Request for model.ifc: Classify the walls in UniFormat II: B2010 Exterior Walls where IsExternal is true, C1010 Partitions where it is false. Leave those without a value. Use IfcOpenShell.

First a look at what the model holds.

```python
import ifcopenshell
import ifcopenshell.util.element

model = ifcopenshell.open("model.ifc")
print(model.schema)
print("classifications:", [c.Name for c in model.by_type("IfcClassification")])
values = [ifcopenshell.util.element.get_pset(e, "Pset_WallCommon", "IsExternal") for e in model.by_type("IfcWall")]
for value in (True, False, None):
    print("IsExternal", value, values.count(value))
```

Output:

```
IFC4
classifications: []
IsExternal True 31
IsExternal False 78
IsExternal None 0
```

```python
import ifcopenshell
import ifcopenshell.api.classification
import ifcopenshell.util.element

model = ifcopenshell.open("model.ifc")

system = ifcopenshell.api.classification.add_classification(model, classification="UniFormat II")

walls = model.by_type("IfcWall")
external = {e: ifcopenshell.util.element.get_pset(e, "Pset_WallCommon", "IsExternal") for e in walls}
for flag, code, name in ((True, "B2010", "Exterior Walls"), (False, "C1010", "Partitions")):
    products = [e for e in walls if external[e] is flag]
    ifcopenshell.api.classification.add_reference(
        model, products=products, classification=system, identification=code, name=name
    )
    print(code, len(products))

model.write("model_edited.ifc")
```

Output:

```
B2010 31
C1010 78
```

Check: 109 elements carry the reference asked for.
